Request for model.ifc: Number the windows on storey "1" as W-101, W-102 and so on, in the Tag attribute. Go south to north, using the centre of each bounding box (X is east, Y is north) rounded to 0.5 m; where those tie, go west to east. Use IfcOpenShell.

First a look at what the model holds.

```python
import ifcopenshell
import ifcopenshell.util.element
import ifcopenshell.util.placement

model = ifcopenshell.open("model.ifc")
print(model.schema)
storey = next(s for s in model.by_type("IfcBuildingStorey") if s.Name == "1")
windows = [e for e in ifcopenshell.util.element.get_decomposition(storey) if e.is_a("IfcWindow")]
for e in sorted(windows, key=lambda e: e.id()):
    origin = ifcopenshell.util.placement.get_local_placement(e.ObjectPlacement)[:3, 3]
    print(e.id(), e.Tag, e.Name, origin.round(2) + 0.0, sep=" | ")
```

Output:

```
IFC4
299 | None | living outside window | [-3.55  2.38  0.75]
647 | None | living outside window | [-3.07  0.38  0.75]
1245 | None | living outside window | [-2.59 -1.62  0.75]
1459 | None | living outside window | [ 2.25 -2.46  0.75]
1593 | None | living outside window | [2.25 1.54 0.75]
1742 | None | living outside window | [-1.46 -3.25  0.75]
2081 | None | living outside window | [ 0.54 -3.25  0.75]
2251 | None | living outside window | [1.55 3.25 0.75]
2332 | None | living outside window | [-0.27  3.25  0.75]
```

```python
import ifcopenshell
import ifcopenshell.geom
import ifcopenshell.util.element
import ifcopenshell.util.shape

model = ifcopenshell.open("model.ifc")
settings = ifcopenshell.geom.settings()
settings.set("use-world-coords", True)


def centre(element):
    shape = ifcopenshell.geom.create_shape(settings, element)
    return ifcopenshell.util.shape.get_bbox_centroid(shape.geometry)


storey = next(s for s in model.by_type("IfcBuildingStorey") if s.Name == "1")
windows = [e for e in ifcopenshell.util.element.get_decomposition(storey) if e.is_a("IfcWindow")]

# Insertion points can sit at a corner or the storey origin, so sort by the geometry (in metres).
centres = {e: centre(e) for e in windows}
windows.sort(key=lambda e: (round(centres[e][1] / 0.5), centres[e][0]))

for i, e in enumerate(windows, start=1):
    number = f"W-1{i:02d}"
    e.Tag = number
    print(e.id(), number)

model.write("model_updated.ifc")
```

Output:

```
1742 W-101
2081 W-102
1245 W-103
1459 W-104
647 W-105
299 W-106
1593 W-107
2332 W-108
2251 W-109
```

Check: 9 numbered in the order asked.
